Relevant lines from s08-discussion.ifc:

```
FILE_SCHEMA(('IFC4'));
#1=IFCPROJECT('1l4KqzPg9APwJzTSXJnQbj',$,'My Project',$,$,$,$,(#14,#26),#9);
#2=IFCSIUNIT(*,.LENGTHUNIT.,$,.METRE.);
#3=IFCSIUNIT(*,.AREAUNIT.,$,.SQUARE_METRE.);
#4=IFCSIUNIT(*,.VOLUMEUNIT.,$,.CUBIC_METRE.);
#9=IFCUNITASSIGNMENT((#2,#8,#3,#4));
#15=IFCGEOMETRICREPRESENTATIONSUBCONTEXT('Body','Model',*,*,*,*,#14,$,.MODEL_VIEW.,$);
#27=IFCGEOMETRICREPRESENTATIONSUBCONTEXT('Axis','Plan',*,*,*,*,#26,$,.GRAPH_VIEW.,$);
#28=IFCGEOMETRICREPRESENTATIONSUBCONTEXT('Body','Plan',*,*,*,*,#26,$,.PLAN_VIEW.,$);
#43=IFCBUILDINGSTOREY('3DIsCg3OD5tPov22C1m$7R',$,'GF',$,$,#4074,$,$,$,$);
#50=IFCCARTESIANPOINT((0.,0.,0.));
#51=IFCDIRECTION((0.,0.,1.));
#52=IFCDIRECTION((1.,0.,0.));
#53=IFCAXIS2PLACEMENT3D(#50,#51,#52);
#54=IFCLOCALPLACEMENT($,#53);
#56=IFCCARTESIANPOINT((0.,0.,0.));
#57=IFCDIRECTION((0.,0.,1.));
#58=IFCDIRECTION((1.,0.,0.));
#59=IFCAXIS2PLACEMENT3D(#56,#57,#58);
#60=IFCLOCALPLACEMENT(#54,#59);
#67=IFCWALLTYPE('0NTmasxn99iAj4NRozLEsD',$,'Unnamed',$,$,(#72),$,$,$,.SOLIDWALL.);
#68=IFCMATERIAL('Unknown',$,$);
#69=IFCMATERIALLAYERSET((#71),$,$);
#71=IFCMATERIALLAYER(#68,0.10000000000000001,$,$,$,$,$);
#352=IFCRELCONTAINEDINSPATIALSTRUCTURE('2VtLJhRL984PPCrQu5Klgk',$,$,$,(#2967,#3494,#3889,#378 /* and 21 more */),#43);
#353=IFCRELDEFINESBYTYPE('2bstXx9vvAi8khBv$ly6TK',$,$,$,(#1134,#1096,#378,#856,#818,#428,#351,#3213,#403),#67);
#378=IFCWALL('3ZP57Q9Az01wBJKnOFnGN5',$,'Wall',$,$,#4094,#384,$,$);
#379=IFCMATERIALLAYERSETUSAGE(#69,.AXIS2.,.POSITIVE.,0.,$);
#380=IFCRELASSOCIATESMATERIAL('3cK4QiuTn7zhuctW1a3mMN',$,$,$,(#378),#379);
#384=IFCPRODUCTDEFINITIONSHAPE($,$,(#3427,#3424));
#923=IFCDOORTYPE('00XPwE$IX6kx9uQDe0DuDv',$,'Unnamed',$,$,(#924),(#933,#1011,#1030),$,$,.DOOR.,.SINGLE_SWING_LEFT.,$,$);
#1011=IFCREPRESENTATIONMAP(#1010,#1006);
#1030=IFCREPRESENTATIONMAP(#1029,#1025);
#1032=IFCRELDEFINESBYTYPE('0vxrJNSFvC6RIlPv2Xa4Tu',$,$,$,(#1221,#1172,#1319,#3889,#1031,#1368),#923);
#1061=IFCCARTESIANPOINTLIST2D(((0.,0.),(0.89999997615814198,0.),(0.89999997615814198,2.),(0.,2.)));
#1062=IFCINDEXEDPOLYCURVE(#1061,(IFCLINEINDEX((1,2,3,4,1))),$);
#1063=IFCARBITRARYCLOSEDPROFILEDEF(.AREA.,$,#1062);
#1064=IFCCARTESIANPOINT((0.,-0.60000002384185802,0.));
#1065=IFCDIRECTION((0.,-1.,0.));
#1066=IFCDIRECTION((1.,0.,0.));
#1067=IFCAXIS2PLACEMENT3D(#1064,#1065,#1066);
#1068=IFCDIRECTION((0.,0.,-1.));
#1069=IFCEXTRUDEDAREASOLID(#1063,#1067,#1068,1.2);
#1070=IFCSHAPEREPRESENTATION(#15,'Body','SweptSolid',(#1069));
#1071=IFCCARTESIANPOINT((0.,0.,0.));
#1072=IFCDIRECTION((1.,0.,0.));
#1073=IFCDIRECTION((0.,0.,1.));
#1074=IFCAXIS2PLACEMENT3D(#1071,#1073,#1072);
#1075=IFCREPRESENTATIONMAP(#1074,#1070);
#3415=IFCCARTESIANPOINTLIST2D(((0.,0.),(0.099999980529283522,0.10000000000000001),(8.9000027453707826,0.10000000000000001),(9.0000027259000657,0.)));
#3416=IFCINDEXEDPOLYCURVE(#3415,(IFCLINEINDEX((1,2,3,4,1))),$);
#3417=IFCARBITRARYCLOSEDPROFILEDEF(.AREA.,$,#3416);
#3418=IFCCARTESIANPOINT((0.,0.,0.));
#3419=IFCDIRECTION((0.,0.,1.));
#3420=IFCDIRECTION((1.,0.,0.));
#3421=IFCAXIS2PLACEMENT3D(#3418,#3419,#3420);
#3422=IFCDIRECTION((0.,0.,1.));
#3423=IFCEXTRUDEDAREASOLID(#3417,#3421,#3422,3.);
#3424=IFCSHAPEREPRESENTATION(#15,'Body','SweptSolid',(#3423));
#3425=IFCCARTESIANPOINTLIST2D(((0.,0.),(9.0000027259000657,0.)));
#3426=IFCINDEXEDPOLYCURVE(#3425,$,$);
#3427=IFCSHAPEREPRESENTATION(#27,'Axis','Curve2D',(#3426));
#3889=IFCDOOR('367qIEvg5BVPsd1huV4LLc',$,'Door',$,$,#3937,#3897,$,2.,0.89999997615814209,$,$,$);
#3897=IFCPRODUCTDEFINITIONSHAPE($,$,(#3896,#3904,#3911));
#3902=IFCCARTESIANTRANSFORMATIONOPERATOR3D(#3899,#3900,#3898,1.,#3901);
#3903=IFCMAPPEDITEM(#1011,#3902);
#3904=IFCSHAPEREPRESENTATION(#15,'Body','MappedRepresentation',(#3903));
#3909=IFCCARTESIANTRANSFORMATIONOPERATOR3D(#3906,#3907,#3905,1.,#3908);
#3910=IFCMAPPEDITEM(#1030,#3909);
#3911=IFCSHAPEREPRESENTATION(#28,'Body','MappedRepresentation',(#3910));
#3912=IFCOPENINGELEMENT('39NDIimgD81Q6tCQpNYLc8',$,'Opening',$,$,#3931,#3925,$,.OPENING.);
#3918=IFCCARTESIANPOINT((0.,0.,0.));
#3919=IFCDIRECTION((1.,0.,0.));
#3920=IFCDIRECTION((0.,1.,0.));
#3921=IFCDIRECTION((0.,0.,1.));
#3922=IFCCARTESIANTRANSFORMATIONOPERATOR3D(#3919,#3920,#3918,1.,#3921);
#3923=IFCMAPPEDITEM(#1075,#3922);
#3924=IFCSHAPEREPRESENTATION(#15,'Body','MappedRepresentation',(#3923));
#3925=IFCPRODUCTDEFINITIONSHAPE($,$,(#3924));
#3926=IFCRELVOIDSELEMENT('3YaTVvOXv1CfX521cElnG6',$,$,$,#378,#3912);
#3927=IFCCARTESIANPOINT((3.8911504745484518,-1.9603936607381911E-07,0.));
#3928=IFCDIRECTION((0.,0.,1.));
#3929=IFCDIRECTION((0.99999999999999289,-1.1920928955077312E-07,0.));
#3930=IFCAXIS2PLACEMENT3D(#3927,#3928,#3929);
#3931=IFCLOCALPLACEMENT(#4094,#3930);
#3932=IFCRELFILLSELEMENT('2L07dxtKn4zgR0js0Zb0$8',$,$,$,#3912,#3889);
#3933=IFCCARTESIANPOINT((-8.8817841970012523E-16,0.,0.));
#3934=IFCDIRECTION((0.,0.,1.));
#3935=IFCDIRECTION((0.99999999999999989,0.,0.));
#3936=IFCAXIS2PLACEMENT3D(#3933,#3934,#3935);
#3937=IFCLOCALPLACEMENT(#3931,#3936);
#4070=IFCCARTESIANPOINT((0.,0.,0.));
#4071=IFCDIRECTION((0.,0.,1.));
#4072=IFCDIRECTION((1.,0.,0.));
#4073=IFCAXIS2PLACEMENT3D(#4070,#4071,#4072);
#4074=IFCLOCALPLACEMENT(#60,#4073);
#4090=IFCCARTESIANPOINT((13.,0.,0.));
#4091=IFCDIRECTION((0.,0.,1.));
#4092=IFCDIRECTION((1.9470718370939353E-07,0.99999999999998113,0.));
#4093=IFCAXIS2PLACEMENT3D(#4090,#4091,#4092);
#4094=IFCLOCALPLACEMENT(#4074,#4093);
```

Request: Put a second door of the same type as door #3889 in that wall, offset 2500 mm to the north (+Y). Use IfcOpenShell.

```python
import ifcopenshell
import ifcopenshell.api.feature
import ifcopenshell.api.geometry
import ifcopenshell.api.root
import ifcopenshell.geom
import ifcopenshell.util.element
import ifcopenshell.util.placement
import ifcopenshell.util.shape
import ifcopenshell.util.unit

model = ifcopenshell.open("s08-discussion.ifc")
unit_scale = ifcopenshell.util.unit.calculate_unit_scale(model)
settings = ifcopenshell.geom.settings()


def volume(element):
    """Net volume in cubic metres, openings subtracted."""
    shape = ifcopenshell.geom.create_shape(settings, element)
    return ifcopenshell.util.shape.get_volume(shape.geometry)


door = model.by_guid("367qIEvg5BVPsd1huV4LLc")
opening = door.FillsVoids[0].RelatingOpeningElement
wall = opening.VoidsElements[0].RelatingBuildingElement
before = volume(wall)
shift = ifcopenshell.util.placement.get_local_placement(wall.ObjectPlacement)[:3, 0] * 2.5 / unit_scale

# copy_class copies the void relationship, type, container and properties, but no geometry.
new_opening = ifcopenshell.api.root.copy_class(model, product=opening)
new_opening.Representation = ifcopenshell.util.element.copy_deep(
    model, opening.Representation, exclude=["IfcGeometricRepresentationContext", "IfcRepresentationMap"]
)
new_door = ifcopenshell.api.root.copy_class(model, product=door)
new_door.Representation = ifcopenshell.util.element.copy_deep(
    model, door.Representation, exclude=["IfcGeometricRepresentationContext", "IfcRepresentationMap"]
)
ifcopenshell.api.feature.add_filling(model, opening=new_opening, element=new_door)

for old, new in ((opening, new_opening), (door, new_door)):
    matrix = ifcopenshell.util.placement.get_local_placement(old.ObjectPlacement)
    matrix[:3, 3] += shift
    ifcopenshell.api.geometry.edit_object_placement(model, product=new, matrix=matrix, is_si=False)

after = volume(wall)

print(f"wall volume {before:.3f} -> {after:.3f} m3")

model.write("s08-discussion_v2.ifc")
```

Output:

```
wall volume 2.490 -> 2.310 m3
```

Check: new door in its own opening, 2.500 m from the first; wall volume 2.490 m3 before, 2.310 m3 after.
